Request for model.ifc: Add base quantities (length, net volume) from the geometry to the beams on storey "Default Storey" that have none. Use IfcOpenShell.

First a look at what the model holds.

```python
import ifcopenshell
import ifcopenshell.util.element
import ifcopenshell.util.unit

model = ifcopenshell.open("model.ifc")
print(model.schema)
for unit_type in ("LENGTHUNIT", "AREAUNIT", "VOLUMEUNIT"):
    print(unit_type, ifcopenshell.util.unit.calculate_unit_scale(model, unit_type))
storey = next(s for s in model.by_type("IfcBuildingStorey") if s.Name == "Default Storey")
beams = [e for e in ifcopenshell.util.element.get_decomposition(storey) if e.is_a("IfcBeam")]
for e in sorted(beams, key=lambda e: e.id()):
    print(e.id(), e.is_a(), e.Name, list(ifcopenshell.util.element.get_psets(e, qtos_only=True)), sep=" | ")
```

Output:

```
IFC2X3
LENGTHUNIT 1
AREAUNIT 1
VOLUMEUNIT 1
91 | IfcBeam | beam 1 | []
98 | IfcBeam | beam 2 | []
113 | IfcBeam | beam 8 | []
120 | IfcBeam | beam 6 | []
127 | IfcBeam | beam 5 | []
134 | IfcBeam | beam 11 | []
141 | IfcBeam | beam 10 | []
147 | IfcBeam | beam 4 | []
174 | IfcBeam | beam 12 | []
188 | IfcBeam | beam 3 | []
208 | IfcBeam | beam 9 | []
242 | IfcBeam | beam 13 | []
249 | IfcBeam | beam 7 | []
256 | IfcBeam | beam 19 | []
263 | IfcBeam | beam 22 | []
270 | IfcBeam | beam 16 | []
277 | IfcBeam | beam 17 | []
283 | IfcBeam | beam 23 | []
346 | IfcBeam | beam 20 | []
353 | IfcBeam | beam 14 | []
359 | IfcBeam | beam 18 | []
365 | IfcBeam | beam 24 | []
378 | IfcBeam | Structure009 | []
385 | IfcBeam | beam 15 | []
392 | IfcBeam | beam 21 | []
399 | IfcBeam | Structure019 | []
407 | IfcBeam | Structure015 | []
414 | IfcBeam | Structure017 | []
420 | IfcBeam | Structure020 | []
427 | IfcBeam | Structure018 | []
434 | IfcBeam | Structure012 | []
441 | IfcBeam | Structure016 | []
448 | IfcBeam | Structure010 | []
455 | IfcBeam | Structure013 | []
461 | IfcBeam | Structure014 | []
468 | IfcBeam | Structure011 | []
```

```python
import ifcopenshell
import ifcopenshell.api.pset
import ifcopenshell.geom
import ifcopenshell.util.element
import ifcopenshell.util.shape
import ifcopenshell.util.unit

model = ifcopenshell.open("model.ifc")
unit_scale = ifcopenshell.util.unit.calculate_unit_scale(model)
volume_scale = ifcopenshell.util.unit.calculate_unit_scale(model, "VOLUMEUNIT")
settings = ifcopenshell.geom.settings()

storey = next(s for s in model.by_type("IfcBuildingStorey") if s.Name == "Default Storey")
beams = [e for e in ifcopenshell.util.element.get_decomposition(storey) if e.is_a("IfcBeam")]

for e in sorted(beams, key=lambda e: e.id()):
    if ifcopenshell.util.element.get_psets(e, qtos_only=True, should_inherit=False):
        continue
    # Geometry comes back in metres, in the element's own axes.
    shape = ifcopenshell.geom.create_shape(settings, e)
    values = {
        "Length": ifcopenshell.util.shape.get_max_xyz(shape.geometry) / unit_scale,
        "NetVolume": ifcopenshell.util.shape.get_volume(shape.geometry) / volume_scale,
    }
    qto = ifcopenshell.api.pset.add_qto(model, product=e, name="BaseQuantities")
    ifcopenshell.api.pset.edit_qto(model, qto=qto, properties=values)
    print(e.id(), {k: round(v, 3) for k, v in values.items()})

model.write("model_rev.ifc")
```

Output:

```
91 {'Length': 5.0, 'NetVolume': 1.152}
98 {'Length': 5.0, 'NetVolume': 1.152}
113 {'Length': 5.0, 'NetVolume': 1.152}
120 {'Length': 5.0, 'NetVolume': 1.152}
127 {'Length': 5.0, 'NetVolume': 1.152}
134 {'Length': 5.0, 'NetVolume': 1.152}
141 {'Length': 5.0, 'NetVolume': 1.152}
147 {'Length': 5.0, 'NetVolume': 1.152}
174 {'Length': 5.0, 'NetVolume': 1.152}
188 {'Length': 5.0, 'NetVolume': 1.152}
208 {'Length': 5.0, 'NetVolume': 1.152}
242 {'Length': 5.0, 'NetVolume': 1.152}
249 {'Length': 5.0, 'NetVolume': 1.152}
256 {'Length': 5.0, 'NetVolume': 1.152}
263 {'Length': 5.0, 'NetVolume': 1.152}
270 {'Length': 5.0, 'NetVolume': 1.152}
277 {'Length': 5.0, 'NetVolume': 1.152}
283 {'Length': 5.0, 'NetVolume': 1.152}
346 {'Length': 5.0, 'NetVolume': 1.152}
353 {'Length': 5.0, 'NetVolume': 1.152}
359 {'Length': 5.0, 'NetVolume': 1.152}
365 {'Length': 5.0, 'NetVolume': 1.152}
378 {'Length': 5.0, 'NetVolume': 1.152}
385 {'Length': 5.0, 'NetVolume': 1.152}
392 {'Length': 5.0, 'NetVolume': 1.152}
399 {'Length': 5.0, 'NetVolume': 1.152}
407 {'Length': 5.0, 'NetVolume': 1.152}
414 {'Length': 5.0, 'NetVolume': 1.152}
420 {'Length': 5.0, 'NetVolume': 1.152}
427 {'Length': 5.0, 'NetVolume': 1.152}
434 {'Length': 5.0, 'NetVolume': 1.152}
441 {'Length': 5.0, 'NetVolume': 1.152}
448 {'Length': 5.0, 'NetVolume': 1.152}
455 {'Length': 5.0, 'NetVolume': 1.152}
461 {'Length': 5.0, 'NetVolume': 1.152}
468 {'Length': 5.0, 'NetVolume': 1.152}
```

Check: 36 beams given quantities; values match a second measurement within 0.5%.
